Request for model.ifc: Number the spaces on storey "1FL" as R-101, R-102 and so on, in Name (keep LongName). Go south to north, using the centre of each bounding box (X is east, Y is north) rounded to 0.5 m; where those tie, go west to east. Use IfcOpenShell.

First a look at what the model holds.

```python
import ifcopenshell
import ifcopenshell.util.element
import ifcopenshell.util.placement

model = ifcopenshell.open("model.ifc")
print(model.schema)
storey = next(s for s in model.by_type("IfcBuildingStorey") if s.Name == "1FL")
spaces = [e for e in ifcopenshell.util.element.get_decomposition(storey) if e.is_a("IfcSpace")]
for e in sorted(spaces, key=lambda e: e.id()):
    origin = ifcopenshell.util.placement.get_local_placement(e.ObjectPlacement)[:3, 3]
    print(e.id(), e.Name, e.LongName, origin.round(2) + 0.0, sep=" | ")
```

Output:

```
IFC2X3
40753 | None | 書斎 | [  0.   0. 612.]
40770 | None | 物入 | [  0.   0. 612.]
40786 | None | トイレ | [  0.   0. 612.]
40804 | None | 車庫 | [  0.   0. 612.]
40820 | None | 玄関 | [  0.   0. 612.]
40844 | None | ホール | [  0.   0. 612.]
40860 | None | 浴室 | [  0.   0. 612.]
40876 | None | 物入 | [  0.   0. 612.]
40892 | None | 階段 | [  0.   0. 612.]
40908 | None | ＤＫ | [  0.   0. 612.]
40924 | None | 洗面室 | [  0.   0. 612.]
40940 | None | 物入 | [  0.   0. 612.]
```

```python
import ifcopenshell
import ifcopenshell.geom
import ifcopenshell.util.element
import ifcopenshell.util.shape

model = ifcopenshell.open("model.ifc")
settings = ifcopenshell.geom.settings()
settings.set("use-world-coords", True)


def centre(element):
    shape = ifcopenshell.geom.create_shape(settings, element)
    return ifcopenshell.util.shape.get_bbox_centroid(shape.geometry)


storey = next(s for s in model.by_type("IfcBuildingStorey") if s.Name == "1FL")
spaces = [e for e in ifcopenshell.util.element.get_decomposition(storey) if e.is_a("IfcSpace")]

# Insertion points can sit at a corner or the storey origin, so sort by the geometry (in metres).
centres = {e: centre(e) for e in spaces}
spaces.sort(key=lambda e: (round(centres[e][1] / 0.5), centres[e][0]))

for i, e in enumerate(spaces, start=1):
    number = f"R-1{i:02d}"
    e.Name = number
    print(e.id(), number)

model.write("model_rev.ifc")
```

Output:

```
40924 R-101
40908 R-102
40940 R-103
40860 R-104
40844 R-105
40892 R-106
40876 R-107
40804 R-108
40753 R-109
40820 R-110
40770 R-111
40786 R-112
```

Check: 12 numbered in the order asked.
